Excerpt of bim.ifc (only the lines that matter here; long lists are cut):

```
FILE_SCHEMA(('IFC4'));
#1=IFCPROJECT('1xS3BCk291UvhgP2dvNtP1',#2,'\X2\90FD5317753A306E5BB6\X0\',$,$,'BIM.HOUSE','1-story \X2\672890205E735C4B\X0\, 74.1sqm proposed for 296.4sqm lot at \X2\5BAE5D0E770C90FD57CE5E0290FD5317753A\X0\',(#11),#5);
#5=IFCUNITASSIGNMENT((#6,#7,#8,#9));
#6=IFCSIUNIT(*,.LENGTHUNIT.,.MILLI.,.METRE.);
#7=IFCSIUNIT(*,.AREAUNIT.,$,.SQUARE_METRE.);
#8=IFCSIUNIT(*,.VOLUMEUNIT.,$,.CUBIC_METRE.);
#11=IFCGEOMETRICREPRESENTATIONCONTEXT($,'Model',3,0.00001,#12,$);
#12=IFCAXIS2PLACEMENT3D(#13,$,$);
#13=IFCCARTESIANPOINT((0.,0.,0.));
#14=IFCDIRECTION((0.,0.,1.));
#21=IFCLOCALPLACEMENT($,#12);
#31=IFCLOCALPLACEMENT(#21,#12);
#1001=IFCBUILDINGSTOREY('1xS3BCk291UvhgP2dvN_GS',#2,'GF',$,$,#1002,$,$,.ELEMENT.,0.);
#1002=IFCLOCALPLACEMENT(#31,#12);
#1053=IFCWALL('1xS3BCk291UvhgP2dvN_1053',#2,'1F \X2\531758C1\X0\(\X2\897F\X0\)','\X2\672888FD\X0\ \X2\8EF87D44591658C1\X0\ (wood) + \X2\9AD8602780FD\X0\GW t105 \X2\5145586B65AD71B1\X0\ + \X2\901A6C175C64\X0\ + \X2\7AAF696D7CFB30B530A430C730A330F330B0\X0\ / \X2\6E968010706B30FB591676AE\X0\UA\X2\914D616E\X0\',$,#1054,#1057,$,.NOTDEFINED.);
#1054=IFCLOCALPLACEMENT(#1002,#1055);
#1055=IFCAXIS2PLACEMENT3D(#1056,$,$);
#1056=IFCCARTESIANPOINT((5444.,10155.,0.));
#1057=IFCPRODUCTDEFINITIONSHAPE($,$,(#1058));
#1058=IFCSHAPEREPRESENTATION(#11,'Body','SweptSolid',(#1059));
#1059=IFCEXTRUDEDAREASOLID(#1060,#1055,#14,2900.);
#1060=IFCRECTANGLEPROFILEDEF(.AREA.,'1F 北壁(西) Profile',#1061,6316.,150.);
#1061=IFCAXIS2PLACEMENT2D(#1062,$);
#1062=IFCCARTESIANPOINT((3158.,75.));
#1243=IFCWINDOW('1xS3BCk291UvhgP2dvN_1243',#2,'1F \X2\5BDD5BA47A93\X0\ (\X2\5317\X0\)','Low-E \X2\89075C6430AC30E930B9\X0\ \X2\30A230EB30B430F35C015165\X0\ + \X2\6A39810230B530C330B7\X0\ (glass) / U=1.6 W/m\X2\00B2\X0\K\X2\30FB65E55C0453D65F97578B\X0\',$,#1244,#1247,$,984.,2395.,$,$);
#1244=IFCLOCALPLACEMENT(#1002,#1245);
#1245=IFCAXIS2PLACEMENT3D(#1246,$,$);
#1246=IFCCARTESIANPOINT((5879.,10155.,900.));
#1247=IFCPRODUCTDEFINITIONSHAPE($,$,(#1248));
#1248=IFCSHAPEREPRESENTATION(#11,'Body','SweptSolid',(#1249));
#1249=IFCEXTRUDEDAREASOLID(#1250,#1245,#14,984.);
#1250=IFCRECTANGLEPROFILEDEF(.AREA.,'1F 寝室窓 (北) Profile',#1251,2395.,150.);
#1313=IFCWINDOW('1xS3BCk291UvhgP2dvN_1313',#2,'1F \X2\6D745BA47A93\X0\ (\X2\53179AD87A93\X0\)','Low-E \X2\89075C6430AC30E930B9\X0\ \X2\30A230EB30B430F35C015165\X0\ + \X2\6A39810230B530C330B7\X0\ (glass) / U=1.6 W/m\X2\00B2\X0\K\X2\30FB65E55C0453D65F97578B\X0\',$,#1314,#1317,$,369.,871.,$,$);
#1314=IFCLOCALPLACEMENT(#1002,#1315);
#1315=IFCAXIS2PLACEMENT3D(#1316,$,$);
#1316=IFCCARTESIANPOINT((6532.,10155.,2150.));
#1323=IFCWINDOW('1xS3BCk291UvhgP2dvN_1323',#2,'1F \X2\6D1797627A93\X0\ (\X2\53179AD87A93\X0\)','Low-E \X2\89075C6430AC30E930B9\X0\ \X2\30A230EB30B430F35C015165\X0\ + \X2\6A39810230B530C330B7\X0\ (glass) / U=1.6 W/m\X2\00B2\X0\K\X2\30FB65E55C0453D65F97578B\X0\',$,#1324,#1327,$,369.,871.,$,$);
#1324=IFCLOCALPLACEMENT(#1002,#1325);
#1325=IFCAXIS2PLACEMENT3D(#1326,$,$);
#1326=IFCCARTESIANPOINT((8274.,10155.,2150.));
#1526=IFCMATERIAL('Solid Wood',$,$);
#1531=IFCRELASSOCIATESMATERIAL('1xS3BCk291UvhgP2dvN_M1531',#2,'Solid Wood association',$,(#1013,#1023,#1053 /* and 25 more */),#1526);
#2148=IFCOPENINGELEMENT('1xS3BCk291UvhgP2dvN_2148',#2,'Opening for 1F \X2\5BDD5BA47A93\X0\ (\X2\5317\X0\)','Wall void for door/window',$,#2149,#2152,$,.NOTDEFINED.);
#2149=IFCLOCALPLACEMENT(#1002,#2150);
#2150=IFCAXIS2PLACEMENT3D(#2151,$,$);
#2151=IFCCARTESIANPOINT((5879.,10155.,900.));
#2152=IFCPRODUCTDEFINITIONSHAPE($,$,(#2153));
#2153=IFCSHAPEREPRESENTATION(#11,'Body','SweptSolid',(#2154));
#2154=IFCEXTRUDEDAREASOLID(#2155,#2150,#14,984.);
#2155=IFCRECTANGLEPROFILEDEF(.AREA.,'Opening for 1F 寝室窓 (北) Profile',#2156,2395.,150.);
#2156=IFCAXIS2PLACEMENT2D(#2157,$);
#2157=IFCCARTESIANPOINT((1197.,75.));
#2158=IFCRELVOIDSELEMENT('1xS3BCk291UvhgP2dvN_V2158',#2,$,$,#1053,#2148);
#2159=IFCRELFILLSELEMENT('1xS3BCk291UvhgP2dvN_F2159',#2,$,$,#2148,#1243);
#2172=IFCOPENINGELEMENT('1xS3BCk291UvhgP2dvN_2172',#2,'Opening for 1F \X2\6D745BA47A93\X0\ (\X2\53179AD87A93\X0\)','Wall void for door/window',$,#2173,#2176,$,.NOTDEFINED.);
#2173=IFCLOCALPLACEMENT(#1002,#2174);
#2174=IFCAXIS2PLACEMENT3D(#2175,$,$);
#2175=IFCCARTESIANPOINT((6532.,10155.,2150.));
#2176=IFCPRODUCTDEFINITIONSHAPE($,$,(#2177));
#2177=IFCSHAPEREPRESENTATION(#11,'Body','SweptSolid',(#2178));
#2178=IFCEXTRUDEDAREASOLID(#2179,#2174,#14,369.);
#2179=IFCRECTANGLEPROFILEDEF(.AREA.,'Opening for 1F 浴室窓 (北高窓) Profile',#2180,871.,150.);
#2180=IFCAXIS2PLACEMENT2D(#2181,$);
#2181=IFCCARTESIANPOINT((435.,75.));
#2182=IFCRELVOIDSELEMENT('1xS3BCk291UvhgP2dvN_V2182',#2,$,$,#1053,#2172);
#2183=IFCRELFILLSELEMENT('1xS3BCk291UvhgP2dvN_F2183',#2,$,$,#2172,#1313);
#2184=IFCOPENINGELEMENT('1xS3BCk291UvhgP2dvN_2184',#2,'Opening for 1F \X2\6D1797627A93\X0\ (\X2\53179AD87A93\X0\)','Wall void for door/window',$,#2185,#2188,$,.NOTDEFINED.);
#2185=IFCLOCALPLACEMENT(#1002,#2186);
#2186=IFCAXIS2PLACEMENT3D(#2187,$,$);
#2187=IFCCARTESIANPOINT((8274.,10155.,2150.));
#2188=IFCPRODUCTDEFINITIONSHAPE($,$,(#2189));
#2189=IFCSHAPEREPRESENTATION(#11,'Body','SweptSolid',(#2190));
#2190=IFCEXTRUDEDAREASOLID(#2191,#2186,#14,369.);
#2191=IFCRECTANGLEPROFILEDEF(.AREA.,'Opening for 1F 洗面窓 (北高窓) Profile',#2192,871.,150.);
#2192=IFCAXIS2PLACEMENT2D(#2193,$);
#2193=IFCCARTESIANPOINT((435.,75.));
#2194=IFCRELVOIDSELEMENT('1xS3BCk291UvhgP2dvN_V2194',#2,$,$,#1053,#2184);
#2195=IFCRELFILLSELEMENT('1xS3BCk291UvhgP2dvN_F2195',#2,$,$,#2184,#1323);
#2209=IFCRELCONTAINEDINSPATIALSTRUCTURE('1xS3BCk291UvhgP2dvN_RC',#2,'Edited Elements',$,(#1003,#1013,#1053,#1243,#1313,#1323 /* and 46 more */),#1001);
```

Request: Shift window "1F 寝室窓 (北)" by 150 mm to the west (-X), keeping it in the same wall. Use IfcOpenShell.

```python
import ifcopenshell
import ifcopenshell.api.geometry
import ifcopenshell.util.placement

model = ifcopenshell.open("bim.ifc")

window = model.by_id(1243)
opening = window.FillsVoids[0].RelatingOpeningElement
wall = opening.VoidsElements[0].RelatingBuildingElement

wall_matrix = ifcopenshell.util.placement.get_local_placement(wall.ObjectPlacement)
shift = wall_matrix[:3, 0] * -150.0
before = ifcopenshell.util.placement.get_local_placement(window.ObjectPlacement)[:3, 3].copy()

# The window is not placed relative to its opening, so move both.
for product in (opening, window):
    matrix = ifcopenshell.util.placement.get_local_placement(product.ObjectPlacement)
    matrix[:3, 3] += shift
    ifcopenshell.api.geometry.edit_object_placement(model, product=product, matrix=matrix, is_si=False)

after = ifcopenshell.util.placement.get_local_placement(window.ObjectPlacement)[:3, 3]
print("window moved by", (after - before).round(3) + 0.0)

model.write("bim_updated.ifc")
```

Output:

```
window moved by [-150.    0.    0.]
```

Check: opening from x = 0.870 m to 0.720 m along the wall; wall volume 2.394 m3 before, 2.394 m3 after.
